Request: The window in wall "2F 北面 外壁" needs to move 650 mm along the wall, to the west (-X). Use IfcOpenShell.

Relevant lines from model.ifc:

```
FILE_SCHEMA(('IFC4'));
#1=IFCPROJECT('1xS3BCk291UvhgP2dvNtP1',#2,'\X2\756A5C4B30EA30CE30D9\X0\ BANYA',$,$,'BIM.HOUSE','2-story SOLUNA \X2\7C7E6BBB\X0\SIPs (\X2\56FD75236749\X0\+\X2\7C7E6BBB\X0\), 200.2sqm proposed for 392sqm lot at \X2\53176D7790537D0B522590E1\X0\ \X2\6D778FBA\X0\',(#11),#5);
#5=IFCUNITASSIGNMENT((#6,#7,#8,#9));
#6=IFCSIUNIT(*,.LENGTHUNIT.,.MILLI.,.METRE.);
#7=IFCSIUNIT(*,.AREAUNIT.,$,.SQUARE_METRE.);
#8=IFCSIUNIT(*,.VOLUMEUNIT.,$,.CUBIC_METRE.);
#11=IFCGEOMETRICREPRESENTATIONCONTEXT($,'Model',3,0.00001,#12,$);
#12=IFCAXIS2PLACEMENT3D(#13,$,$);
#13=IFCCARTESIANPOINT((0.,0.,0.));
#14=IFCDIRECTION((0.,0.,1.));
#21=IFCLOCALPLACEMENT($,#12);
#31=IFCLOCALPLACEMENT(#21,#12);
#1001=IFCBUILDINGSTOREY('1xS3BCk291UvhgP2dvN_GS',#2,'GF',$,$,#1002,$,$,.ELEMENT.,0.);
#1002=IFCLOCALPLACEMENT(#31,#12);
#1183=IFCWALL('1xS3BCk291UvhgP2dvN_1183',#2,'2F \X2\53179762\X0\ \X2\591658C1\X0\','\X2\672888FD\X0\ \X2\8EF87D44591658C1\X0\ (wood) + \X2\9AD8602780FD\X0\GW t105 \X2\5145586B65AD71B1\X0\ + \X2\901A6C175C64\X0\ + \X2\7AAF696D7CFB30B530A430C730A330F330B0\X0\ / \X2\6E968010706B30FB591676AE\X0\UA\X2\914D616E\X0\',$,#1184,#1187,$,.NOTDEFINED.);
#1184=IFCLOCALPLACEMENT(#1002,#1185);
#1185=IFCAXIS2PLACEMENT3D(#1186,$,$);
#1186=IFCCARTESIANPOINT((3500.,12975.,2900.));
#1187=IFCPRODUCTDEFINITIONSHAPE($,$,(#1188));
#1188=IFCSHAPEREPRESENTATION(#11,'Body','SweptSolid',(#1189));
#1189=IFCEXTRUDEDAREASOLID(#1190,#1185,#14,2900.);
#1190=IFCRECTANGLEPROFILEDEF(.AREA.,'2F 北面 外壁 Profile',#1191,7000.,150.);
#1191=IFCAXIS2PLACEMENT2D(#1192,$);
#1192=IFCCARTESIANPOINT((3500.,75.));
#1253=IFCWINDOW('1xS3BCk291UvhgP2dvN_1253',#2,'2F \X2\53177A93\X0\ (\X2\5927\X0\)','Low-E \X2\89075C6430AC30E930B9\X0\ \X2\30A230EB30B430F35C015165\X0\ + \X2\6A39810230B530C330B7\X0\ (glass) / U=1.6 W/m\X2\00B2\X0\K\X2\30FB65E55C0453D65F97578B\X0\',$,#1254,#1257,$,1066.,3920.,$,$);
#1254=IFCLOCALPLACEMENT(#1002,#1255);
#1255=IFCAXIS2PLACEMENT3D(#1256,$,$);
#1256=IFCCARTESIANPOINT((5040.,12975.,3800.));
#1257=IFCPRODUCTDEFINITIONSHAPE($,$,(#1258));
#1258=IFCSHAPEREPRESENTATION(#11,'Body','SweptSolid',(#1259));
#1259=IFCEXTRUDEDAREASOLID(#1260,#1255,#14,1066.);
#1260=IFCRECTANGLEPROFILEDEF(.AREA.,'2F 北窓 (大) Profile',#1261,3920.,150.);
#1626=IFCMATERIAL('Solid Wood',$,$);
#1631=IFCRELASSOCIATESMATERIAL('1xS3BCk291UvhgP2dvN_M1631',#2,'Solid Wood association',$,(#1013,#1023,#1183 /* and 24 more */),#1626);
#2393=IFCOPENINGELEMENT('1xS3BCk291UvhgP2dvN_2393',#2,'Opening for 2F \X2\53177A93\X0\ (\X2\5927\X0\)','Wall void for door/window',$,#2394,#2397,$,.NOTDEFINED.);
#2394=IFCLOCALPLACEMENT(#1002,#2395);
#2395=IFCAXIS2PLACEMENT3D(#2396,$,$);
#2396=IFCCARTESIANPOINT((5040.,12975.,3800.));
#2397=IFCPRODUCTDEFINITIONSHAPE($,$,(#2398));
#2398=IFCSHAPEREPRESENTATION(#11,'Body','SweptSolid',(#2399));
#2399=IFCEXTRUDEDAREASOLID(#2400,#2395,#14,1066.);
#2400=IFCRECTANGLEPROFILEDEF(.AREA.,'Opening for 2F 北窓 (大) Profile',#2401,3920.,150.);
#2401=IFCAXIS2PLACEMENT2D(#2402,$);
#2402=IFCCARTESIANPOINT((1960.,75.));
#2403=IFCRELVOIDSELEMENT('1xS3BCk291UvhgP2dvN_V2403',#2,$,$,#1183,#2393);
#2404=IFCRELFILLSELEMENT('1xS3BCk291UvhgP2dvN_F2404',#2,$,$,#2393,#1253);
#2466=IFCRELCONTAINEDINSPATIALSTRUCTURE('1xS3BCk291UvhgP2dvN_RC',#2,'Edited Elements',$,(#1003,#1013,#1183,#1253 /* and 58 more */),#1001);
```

```python
import ifcopenshell
import ifcopenshell.api.geometry
import ifcopenshell.util.placement

model = ifcopenshell.open("model.ifc")

window = model.by_guid("1xS3BCk291UvhgP2dvN_1253")
opening = window.FillsVoids[0].RelatingOpeningElement
wall = opening.VoidsElements[0].RelatingBuildingElement

wall_matrix = ifcopenshell.util.placement.get_local_placement(wall.ObjectPlacement)
shift = wall_matrix[:3, 0] * -650.0
before = ifcopenshell.util.placement.get_local_placement(window.ObjectPlacement)[:3, 3].copy()

# The window is not placed relative to its opening, so move both.
for product in (opening, window):
    matrix = ifcopenshell.util.placement.get_local_placement(product.ObjectPlacement)
    matrix[:3, 3] += shift
    ifcopenshell.api.geometry.edit_object_placement(model, product=product, matrix=matrix, is_si=False)

after = ifcopenshell.util.placement.get_local_placement(window.ObjectPlacement)[:3, 3]
print("window moved by", (after - before).round(3) + 0.0)

model.write("model_edited.ifc")
```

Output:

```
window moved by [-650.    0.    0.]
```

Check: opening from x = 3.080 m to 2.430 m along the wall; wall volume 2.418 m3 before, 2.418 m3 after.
